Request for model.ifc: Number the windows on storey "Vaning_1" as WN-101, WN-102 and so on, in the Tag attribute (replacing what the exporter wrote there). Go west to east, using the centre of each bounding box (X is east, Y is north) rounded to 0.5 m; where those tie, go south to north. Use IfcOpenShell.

First a look at what the model holds.

```python
import ifcopenshell
import ifcopenshell.util.element
import ifcopenshell.util.placement

model = ifcopenshell.open("model.ifc")
print(model.schema)
storey = next(s for s in model.by_type("IfcBuildingStorey") if s.Name == "Vaning_1")
windows = [e for e in ifcopenshell.util.element.get_decomposition(storey) if e.is_a("IfcWindow")]
for e in sorted(windows, key=lambda e: e.id()):
    origin = ifcopenshell.util.placement.get_local_placement(e.ObjectPlacement)[:3, 3]
    print(e.id(), e.Tag, e.Name, origin.round(2) + 0.0, sep=" | ")
```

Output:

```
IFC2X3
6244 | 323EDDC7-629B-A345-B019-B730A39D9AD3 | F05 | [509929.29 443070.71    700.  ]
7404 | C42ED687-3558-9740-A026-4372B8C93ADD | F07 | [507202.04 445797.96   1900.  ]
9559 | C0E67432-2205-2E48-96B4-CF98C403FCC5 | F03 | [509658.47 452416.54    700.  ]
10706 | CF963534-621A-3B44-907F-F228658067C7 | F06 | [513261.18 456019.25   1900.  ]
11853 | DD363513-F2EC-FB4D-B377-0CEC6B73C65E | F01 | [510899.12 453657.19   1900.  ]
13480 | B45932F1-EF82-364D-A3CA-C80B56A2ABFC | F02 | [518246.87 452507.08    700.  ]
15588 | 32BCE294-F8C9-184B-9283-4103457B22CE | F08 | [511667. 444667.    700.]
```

```python
import ifcopenshell
import ifcopenshell.geom
import ifcopenshell.util.element
import ifcopenshell.util.shape

model = ifcopenshell.open("model.ifc")
settings = ifcopenshell.geom.settings()
settings.set("use-world-coords", True)


def centre(element):
    shape = ifcopenshell.geom.create_shape(settings, element)
    return ifcopenshell.util.shape.get_bbox_centroid(shape.geometry)


storey = next(s for s in model.by_type("IfcBuildingStorey") if s.Name == "Vaning_1")
windows = [e for e in ifcopenshell.util.element.get_decomposition(storey) if e.is_a("IfcWindow")]

# Insertion points can sit at a corner or the storey origin, so sort by the geometry (in metres).
centres = {e: centre(e) for e in windows}
windows.sort(key=lambda e: (round(centres[e][0] / 0.5), centres[e][1]))

for i, e in enumerate(windows, start=1):
    number = f"WN-1{i:02d}"
    e.Tag = number
    print(e.id(), number)

model.write("model_v2.ifc")
```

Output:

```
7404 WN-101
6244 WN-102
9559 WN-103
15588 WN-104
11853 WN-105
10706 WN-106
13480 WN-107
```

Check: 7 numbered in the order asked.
